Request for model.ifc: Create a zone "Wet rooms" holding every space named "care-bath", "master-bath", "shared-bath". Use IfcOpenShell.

First a look at what the model holds.

```python
import ifcopenshell

model = ifcopenshell.open("model.ifc")
print(model.schema)
seen = {}
for space in model.by_type("IfcSpace"):
    seen[space.LongName] = seen.get(space.LongName, 0) + 1
for name, count in sorted(seen.items(), key=str):
    print(count, "x", name)
print("zones:", [z.Name for z in model.by_type("IfcZone")][:20])
```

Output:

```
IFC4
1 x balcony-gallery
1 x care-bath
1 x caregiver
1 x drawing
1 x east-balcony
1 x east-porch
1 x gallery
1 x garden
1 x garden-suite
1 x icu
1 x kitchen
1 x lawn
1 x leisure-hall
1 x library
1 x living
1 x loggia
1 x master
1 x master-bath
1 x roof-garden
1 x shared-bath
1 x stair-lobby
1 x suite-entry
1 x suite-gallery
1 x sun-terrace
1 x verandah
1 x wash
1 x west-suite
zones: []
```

```python
import ifcopenshell
import ifcopenshell.api.group
import ifcopenshell.api.root

model = ifcopenshell.open("model.ifc")

names = {"care-bath", "master-bath", "shared-bath"}
spaces = [s for s in model.by_type("IfcSpace") if s.LongName in names]

zone = ifcopenshell.api.root.create_entity(model, ifc_class="IfcZone", name="Wet rooms")
ifcopenshell.api.group.assign_group(model, products=spaces, group=zone)
print(len(spaces), "spaces in", zone.Name)

model.write("model-out.ifc")
```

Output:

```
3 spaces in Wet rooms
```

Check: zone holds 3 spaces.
